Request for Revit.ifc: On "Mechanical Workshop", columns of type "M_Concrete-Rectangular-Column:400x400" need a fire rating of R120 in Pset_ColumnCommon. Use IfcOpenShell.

First a look at what the model holds.

```python
import ifcopenshell
import ifcopenshell.util.element

model = ifcopenshell.open("Revit.ifc")
print(model.schema)
storey = next(s for s in model.by_type("IfcBuildingStorey") if s.Name == "Mechanical Workshop")
columns = [e for e in ifcopenshell.util.element.get_decomposition(storey) if e.is_a("IfcColumn")]
seen = {}
for e in columns:
    element_type = ifcopenshell.util.element.get_type(e)
    key = (element_type.Name if element_type != e and element_type else None, ifcopenshell.util.element.get_pset(e, "Pset_ColumnCommon", "FireRating"))
    seen[key] = seen.get(key, 0) + 1
for (name, value), count in sorted(seen.items(), key=str):
    print(count, "x", name, "|", value)
```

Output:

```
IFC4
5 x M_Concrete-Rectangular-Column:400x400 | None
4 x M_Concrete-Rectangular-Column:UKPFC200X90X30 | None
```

```python
import ifcopenshell
import ifcopenshell.api.pset
import ifcopenshell.util.element

model = ifcopenshell.open("Revit.ifc")

storey = next(s for s in model.by_type("IfcBuildingStorey") if s.Name == "Mechanical Workshop")
columns = [e for e in ifcopenshell.util.element.get_decomposition(storey) if e.is_a("IfcColumn")]

count = 0
for e in columns:
    element_type = ifcopenshell.util.element.get_type(e)
    if element_type in (None, e) or element_type.Name != "M_Concrete-Rectangular-Column:400x400":
        continue
    # add_pset returns the element's existing set when there is one.
    pset = ifcopenshell.api.pset.add_pset(model, product=e, name="Pset_ColumnCommon")
    ifcopenshell.api.pset.edit_pset(model, pset=pset, properties={"FireRating": "R120"})
    count += 1

print(count, "columns updated")

model.write("Revit_rev.ifc")
```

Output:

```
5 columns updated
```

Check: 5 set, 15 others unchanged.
